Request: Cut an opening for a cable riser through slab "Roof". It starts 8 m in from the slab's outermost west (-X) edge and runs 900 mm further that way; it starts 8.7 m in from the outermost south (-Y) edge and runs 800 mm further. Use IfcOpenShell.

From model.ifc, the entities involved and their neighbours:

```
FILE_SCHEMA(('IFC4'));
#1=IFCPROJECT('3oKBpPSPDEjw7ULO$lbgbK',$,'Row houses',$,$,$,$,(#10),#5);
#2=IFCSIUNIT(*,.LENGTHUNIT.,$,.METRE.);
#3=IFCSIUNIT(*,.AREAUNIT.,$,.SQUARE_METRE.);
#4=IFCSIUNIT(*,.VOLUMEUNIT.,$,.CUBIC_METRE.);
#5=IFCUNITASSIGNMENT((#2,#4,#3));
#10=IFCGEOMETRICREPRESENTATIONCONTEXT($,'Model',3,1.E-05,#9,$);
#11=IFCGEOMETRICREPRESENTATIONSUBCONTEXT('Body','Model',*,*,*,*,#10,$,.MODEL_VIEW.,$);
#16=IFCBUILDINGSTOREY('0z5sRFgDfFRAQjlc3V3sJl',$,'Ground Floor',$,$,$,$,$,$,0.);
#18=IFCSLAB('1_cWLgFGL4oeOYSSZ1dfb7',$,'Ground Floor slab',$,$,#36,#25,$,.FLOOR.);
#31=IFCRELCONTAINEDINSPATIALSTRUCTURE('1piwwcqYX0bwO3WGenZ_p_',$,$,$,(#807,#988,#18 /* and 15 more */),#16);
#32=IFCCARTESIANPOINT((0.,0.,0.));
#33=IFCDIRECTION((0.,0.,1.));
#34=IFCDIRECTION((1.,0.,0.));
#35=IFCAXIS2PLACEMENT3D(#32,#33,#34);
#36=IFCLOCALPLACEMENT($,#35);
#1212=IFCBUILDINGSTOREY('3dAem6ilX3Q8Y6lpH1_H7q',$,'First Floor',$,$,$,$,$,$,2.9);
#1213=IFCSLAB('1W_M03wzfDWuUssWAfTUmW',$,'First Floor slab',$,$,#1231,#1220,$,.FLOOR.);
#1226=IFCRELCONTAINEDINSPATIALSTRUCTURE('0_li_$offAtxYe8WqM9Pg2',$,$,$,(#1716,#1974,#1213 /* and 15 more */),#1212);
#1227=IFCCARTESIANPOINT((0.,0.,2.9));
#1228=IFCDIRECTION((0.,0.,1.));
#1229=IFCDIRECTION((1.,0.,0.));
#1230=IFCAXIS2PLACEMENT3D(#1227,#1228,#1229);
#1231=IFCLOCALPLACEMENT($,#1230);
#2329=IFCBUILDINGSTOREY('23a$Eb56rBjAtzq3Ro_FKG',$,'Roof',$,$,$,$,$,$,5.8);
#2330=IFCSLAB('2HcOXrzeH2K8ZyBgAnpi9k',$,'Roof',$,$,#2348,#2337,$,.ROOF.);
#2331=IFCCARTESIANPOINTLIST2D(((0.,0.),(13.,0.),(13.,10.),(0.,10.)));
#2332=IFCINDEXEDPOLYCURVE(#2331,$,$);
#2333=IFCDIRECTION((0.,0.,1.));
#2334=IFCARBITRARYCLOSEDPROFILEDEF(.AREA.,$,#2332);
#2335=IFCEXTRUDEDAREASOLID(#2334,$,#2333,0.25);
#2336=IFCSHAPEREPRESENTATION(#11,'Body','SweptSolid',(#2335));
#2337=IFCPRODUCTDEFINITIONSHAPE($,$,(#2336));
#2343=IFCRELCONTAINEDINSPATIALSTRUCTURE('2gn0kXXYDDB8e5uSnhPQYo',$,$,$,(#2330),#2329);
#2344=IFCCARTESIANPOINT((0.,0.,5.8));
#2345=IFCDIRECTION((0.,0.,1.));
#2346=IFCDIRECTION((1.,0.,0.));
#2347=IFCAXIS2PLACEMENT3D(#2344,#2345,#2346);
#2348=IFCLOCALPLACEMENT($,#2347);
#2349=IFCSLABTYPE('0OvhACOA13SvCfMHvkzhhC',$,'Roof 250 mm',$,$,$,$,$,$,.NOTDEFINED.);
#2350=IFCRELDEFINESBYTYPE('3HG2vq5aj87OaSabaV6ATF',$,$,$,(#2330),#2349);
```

```python
import numpy as np
import ifcopenshell
import ifcopenshell.api.feature
import ifcopenshell.api.geometry
import ifcopenshell.api.root
import ifcopenshell.geom
import ifcopenshell.util.placement
import ifcopenshell.util.representation
import ifcopenshell.util.shape
import ifcopenshell.util.unit

model = ifcopenshell.open("model.ifc")
unit_scale = ifcopenshell.util.unit.calculate_unit_scale(model)
settings = ifcopenshell.geom.settings()


def volume(element):
    """Net volume in cubic metres, openings subtracted."""
    shape = ifcopenshell.geom.create_shape(settings, element)
    return ifcopenshell.util.shape.get_volume(shape.geometry)


slab = model.by_guid("2HcOXrzeH2K8ZyBgAnpi9k")
before = volume(slab)

# Extent in the slab's own axes, in metres. The edges named are its -X and -Y sides.
slab_shape = ifcopenshell.geom.create_shape(settings, slab)
vertices = ifcopenshell.util.shape.get_vertices(slab_shape.geometry)
x_min, y_min, bottom = vertices.min(axis=0)
top = vertices[:, 2].max()

opening = ifcopenshell.api.root.create_entity(model, ifc_class="IfcOpeningElement", name="Cable riser opening", predefined_type="OPENING")
context = ifcopenshell.util.representation.get_context(model, "Model", "Body", "MODEL_VIEW")
width, depth = 0.9, 0.8
outline = [(0.0, 0.0), (width, 0.0), (width, depth), (0.0, depth), (0.0, 0.0)]
# Overshoot both faces by 50 mm so the cut is clean.
shape = ifcopenshell.api.geometry.add_slab_representation(
    model, context=context, depth=top - bottom + 0.1, polyline=outline
)
ifcopenshell.api.geometry.assign_representation(model, product=opening, representation=shape)

matrix = ifcopenshell.util.placement.get_local_placement(slab.ObjectPlacement)
matrix[:, 3] = matrix @ np.append(np.array([x_min + 8, y_min + 8.7, bottom - 0.05]) / unit_scale, 1.0)
ifcopenshell.api.geometry.edit_object_placement(model, product=opening, matrix=matrix, is_si=False)
ifcopenshell.api.feature.add_feature(model, feature=opening, element=slab)

after = volume(slab)

print(f"slab volume {before:.3f} -> {after:.3f} m3")

model.write("model_rev.ifc")
```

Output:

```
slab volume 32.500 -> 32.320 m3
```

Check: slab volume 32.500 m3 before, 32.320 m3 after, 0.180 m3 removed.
